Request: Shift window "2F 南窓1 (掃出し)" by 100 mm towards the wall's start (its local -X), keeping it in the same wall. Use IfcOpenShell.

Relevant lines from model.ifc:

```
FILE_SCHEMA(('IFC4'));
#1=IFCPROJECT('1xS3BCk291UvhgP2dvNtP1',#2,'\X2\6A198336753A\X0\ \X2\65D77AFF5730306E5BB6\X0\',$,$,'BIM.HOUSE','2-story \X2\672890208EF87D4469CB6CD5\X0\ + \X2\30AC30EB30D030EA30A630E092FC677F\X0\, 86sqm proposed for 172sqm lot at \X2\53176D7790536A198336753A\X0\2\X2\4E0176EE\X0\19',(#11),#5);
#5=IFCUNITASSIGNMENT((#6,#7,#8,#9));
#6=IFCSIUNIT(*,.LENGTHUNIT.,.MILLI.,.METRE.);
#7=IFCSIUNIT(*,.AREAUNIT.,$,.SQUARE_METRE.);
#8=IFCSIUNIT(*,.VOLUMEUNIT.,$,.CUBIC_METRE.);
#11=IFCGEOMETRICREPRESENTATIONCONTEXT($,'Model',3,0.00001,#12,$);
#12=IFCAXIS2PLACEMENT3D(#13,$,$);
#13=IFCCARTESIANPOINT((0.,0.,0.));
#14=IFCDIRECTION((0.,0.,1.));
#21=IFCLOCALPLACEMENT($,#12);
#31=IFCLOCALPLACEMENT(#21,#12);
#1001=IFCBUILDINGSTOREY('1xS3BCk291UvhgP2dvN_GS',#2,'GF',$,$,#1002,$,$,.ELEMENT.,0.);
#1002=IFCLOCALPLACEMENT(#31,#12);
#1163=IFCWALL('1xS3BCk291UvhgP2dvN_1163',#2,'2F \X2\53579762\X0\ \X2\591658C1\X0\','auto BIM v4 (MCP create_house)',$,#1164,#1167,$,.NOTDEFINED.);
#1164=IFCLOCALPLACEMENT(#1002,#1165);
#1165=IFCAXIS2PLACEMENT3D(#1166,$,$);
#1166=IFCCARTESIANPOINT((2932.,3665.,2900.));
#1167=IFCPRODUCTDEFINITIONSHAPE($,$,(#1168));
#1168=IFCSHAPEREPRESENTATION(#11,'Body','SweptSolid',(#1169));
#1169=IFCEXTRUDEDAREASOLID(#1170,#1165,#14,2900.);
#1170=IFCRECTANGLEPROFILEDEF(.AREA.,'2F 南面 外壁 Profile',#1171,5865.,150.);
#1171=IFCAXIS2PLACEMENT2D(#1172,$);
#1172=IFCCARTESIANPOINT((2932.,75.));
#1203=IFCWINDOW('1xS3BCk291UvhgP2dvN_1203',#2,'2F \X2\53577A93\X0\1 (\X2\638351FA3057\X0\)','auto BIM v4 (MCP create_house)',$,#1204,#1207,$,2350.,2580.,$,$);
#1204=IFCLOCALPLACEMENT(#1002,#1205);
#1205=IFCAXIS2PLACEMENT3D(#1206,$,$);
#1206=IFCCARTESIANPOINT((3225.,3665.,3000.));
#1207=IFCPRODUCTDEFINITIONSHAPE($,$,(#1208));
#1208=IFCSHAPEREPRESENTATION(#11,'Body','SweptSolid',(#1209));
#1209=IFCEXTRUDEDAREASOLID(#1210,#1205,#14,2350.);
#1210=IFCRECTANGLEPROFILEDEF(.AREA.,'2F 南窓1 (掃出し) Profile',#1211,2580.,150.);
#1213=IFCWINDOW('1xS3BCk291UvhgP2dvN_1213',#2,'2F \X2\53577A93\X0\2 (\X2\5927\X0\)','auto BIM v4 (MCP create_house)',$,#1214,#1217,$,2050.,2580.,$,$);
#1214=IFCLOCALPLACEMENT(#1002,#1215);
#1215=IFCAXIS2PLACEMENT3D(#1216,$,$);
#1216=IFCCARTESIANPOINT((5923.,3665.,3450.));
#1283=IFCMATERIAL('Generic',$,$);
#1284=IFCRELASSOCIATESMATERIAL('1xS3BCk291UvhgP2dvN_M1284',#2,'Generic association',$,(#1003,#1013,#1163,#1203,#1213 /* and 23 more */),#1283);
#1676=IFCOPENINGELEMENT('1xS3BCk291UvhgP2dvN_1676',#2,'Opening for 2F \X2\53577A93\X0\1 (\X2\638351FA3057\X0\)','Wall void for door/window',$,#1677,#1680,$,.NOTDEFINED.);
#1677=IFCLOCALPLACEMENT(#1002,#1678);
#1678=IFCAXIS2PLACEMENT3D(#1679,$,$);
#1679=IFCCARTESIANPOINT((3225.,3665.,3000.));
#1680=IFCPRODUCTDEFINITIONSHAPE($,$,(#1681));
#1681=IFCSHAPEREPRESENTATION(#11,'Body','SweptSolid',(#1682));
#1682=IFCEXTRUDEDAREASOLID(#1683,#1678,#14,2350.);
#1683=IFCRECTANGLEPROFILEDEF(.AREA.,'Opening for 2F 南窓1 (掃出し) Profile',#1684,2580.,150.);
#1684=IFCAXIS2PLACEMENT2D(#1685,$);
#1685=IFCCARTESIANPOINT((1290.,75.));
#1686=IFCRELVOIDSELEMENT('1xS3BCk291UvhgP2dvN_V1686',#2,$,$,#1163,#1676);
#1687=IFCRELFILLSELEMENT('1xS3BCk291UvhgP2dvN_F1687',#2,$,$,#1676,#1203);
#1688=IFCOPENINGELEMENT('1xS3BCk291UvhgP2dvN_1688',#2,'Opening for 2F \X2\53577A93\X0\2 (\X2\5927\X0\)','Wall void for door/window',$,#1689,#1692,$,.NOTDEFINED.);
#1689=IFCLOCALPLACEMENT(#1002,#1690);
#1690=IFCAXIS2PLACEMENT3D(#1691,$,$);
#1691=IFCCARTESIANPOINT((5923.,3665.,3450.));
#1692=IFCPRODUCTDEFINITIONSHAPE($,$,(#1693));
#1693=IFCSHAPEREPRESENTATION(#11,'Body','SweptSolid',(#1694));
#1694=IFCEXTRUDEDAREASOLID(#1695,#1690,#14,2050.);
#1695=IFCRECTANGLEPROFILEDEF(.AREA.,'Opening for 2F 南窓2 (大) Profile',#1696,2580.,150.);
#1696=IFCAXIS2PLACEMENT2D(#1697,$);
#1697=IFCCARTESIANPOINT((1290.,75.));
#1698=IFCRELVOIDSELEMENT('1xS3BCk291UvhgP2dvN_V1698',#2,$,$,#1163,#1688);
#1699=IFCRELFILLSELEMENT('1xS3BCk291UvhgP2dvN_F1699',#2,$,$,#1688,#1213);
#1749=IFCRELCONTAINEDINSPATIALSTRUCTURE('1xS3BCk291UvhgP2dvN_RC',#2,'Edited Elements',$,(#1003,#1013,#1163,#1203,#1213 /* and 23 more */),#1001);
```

```python
import ifcopenshell
import ifcopenshell.api.geometry
import ifcopenshell.util.placement
import ifcopenshell.util.unit

model = ifcopenshell.open("model.ifc")
unit_scale = ifcopenshell.util.unit.calculate_unit_scale(model)

window = model.by_guid("1xS3BCk291UvhgP2dvN_1203")
opening = window.FillsVoids[0].RelatingOpeningElement
wall = opening.VoidsElements[0].RelatingBuildingElement

wall_matrix = ifcopenshell.util.placement.get_local_placement(wall.ObjectPlacement)
shift = wall_matrix[:3, 0] * -0.1 / unit_scale
before = ifcopenshell.util.placement.get_local_placement(window.ObjectPlacement)[:3, 3].copy()

# The window is not placed relative to its opening, so move both.
for product in (opening, window):
    matrix = ifcopenshell.util.placement.get_local_placement(product.ObjectPlacement)
    matrix[:3, 3] += shift
    ifcopenshell.api.geometry.edit_object_placement(model, product=product, matrix=matrix, is_si=False)

after = ifcopenshell.util.placement.get_local_placement(window.ObjectPlacement)[:3, 3]
print("window moved by", (after - before).round(3) + 0.0)

model.write("model_v2.ifc")
```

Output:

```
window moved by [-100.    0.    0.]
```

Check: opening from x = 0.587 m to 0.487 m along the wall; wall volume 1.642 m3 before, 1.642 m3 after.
